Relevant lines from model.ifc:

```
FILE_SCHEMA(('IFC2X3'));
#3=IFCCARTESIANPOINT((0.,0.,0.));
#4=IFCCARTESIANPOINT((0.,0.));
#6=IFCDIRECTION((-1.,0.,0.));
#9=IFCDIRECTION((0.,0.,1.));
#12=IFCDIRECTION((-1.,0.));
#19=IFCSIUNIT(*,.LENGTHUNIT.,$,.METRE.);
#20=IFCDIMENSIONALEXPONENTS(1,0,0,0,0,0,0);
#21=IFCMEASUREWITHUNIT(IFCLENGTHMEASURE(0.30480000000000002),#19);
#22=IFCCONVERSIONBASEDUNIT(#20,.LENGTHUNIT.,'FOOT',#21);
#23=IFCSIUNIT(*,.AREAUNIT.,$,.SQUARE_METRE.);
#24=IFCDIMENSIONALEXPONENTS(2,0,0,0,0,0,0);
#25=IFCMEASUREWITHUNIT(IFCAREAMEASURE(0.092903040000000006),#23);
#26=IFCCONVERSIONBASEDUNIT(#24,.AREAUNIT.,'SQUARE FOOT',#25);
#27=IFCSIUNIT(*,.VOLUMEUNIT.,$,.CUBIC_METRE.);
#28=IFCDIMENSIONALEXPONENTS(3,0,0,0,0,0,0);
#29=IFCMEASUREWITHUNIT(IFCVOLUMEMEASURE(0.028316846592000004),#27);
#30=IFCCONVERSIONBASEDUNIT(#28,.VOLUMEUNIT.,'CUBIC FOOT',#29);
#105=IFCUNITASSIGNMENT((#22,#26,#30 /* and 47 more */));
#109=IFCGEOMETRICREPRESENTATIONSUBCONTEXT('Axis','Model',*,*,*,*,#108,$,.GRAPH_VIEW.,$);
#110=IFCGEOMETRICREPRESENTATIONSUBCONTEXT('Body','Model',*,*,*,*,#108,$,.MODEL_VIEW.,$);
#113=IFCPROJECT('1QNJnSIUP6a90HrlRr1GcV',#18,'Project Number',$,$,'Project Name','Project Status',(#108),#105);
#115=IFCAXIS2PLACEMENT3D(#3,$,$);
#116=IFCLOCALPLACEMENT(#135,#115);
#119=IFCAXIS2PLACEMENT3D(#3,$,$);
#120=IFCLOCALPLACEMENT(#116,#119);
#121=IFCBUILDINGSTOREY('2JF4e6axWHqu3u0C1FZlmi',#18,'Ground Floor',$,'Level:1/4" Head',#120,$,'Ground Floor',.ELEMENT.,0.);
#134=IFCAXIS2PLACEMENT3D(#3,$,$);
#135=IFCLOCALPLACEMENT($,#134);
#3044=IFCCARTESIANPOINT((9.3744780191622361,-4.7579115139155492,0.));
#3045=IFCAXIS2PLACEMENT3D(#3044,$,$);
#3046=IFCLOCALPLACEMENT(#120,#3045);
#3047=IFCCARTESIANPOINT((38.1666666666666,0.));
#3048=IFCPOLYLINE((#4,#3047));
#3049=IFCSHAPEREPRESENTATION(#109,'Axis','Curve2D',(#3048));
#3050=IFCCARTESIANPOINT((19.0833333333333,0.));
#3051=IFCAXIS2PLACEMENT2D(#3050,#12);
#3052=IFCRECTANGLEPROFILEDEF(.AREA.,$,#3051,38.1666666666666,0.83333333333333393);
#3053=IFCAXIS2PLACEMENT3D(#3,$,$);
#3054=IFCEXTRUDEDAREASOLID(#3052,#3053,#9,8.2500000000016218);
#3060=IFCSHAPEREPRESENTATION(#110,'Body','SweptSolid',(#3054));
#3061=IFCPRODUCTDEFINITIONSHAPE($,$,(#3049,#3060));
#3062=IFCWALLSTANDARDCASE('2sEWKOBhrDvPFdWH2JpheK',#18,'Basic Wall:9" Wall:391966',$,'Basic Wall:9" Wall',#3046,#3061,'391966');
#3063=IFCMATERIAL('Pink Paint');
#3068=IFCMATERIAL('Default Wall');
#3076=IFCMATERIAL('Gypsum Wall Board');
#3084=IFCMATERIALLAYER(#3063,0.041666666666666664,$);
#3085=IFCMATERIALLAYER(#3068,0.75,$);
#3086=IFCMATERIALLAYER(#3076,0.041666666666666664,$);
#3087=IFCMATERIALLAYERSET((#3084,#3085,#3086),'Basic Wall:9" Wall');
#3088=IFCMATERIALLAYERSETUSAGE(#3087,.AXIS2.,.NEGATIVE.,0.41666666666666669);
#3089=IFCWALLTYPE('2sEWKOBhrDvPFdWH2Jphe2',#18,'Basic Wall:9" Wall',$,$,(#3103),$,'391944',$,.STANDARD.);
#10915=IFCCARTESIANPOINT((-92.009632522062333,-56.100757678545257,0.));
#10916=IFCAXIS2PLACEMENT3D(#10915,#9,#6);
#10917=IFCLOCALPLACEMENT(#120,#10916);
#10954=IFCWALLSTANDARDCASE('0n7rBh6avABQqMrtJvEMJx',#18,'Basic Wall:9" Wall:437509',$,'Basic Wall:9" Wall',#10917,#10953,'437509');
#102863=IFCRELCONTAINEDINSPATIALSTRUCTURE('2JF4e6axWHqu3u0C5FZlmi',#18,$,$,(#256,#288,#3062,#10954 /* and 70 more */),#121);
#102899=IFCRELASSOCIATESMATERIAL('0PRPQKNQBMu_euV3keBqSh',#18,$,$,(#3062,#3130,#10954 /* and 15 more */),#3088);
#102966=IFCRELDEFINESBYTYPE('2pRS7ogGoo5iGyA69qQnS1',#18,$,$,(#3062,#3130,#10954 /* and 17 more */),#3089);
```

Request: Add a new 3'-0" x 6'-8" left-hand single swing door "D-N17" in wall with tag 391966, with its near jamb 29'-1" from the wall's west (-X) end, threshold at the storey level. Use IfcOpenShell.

```python
import numpy as np
import ifcopenshell
import ifcopenshell.api.feature
import ifcopenshell.api.geometry
import ifcopenshell.api.root
import ifcopenshell.api.spatial
import ifcopenshell.api.type
import ifcopenshell.geom
import ifcopenshell.util.element
import ifcopenshell.util.placement
import ifcopenshell.util.representation
import ifcopenshell.util.shape
import ifcopenshell.util.unit

model = ifcopenshell.open("model.ifc")
unit_scale = ifcopenshell.util.unit.calculate_unit_scale(model)
settings = ifcopenshell.geom.settings()


def volume(element):
    """Net volume in cubic metres, openings subtracted."""
    shape = ifcopenshell.geom.create_shape(settings, element)
    return ifcopenshell.util.shape.get_volume(shape.geometry)


wall = model.by_guid("2sEWKOBhrDvPFdWH2JpheK")
storey = ifcopenshell.util.element.get_container(wall, ifc_class="IfcBuildingStorey")
context = ifcopenshell.util.representation.get_context(model, "Model", "Body", "MODEL_VIEW")
before = volume(wall)

width, height, from_end, sill = 0.9144, 2.032, 8.8646, 0.0  # metres

# The wall runs along its own X axis, and the end named is its -X end.
wall_shape = ifcopenshell.geom.create_shape(settings, wall)
x, y, z = ifcopenshell.util.shape.get_vertices(wall_shape.geometry).T
start = x.min() + from_end
face, thickness = float(y.min()), float(y.max() - y.min())
wall_matrix = ifcopenshell.util.placement.get_local_placement(wall.ObjectPlacement)
level = ifcopenshell.util.placement.get_local_placement(storey.ObjectPlacement)[2, 3]


def in_wall(x, y):
    """Placement at x, y metres in the wall's axes, at sill height."""
    matrix = wall_matrix.copy()
    matrix[:, 3] = wall_matrix @ np.array([x / unit_scale, y / unit_scale, 0.0, 1.0])
    matrix[2, 3] = level + sill / unit_scale
    return matrix


# Opening: a box that overshoots both wall faces by 50 mm.
opening = ifcopenshell.api.root.create_entity(model, ifc_class="IfcOpeningElement")
box = ifcopenshell.api.geometry.add_wall_representation(
    model, context=context, length=width, height=height, thickness=thickness + 0.1
)
ifcopenshell.api.geometry.assign_representation(model, product=opening, representation=box)
ifcopenshell.api.geometry.edit_object_placement(model, product=opening, matrix=in_wall(start, face - 0.05), is_si=False)
ifcopenshell.api.feature.add_feature(model, feature=opening, element=wall)

door = ifcopenshell.api.root.create_entity(model, ifc_class="IfcDoor", name="D-N17")
door.OverallWidth, door.OverallHeight = width / unit_scale, height / unit_scale
body = ifcopenshell.api.geometry.add_door_representation(
    model,
    context=context,
    overall_width=door.OverallWidth,
    overall_height=door.OverallHeight,
    operation_type="SINGLE_SWING_LEFT",
    lining_properties={"LiningDepth": thickness / unit_scale, "ThresholdDepth": thickness / unit_scale},
)
ifcopenshell.api.geometry.assign_representation(model, product=door, representation=body)
ifcopenshell.api.spatial.assign_container(model, products=[door], relating_structure=storey)
fills = ifcopenshell.api.feature.add_filling(model, opening=opening, element=door)
fills.OwnerHistory = door.OwnerHistory  # required in IFC2X3

# IFC2X3 keeps the operation on the door style.
style = ifcopenshell.api.root.create_entity(model, ifc_class="IfcDoorStyle", name="D-N17")
style.OperationType, style.ConstructionType = "SINGLE_SWING_LEFT", "NOTDEFINED"
style.ParameterTakesPrecedence = style.Sizeable = False
ifcopenshell.api.type.assign_type(model, related_objects=[door], relating_type=style)

# The lining spans the wall, so the door starts at the wall face.
ifcopenshell.api.geometry.edit_object_placement(model, product=door, matrix=in_wall(start, face), is_si=False)

after = volume(wall)

print(f"wall volume {before:.3f} -> {after:.3f} m3")

model.write("model_rev.ifc")
```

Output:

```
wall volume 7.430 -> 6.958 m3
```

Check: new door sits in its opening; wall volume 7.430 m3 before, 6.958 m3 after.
